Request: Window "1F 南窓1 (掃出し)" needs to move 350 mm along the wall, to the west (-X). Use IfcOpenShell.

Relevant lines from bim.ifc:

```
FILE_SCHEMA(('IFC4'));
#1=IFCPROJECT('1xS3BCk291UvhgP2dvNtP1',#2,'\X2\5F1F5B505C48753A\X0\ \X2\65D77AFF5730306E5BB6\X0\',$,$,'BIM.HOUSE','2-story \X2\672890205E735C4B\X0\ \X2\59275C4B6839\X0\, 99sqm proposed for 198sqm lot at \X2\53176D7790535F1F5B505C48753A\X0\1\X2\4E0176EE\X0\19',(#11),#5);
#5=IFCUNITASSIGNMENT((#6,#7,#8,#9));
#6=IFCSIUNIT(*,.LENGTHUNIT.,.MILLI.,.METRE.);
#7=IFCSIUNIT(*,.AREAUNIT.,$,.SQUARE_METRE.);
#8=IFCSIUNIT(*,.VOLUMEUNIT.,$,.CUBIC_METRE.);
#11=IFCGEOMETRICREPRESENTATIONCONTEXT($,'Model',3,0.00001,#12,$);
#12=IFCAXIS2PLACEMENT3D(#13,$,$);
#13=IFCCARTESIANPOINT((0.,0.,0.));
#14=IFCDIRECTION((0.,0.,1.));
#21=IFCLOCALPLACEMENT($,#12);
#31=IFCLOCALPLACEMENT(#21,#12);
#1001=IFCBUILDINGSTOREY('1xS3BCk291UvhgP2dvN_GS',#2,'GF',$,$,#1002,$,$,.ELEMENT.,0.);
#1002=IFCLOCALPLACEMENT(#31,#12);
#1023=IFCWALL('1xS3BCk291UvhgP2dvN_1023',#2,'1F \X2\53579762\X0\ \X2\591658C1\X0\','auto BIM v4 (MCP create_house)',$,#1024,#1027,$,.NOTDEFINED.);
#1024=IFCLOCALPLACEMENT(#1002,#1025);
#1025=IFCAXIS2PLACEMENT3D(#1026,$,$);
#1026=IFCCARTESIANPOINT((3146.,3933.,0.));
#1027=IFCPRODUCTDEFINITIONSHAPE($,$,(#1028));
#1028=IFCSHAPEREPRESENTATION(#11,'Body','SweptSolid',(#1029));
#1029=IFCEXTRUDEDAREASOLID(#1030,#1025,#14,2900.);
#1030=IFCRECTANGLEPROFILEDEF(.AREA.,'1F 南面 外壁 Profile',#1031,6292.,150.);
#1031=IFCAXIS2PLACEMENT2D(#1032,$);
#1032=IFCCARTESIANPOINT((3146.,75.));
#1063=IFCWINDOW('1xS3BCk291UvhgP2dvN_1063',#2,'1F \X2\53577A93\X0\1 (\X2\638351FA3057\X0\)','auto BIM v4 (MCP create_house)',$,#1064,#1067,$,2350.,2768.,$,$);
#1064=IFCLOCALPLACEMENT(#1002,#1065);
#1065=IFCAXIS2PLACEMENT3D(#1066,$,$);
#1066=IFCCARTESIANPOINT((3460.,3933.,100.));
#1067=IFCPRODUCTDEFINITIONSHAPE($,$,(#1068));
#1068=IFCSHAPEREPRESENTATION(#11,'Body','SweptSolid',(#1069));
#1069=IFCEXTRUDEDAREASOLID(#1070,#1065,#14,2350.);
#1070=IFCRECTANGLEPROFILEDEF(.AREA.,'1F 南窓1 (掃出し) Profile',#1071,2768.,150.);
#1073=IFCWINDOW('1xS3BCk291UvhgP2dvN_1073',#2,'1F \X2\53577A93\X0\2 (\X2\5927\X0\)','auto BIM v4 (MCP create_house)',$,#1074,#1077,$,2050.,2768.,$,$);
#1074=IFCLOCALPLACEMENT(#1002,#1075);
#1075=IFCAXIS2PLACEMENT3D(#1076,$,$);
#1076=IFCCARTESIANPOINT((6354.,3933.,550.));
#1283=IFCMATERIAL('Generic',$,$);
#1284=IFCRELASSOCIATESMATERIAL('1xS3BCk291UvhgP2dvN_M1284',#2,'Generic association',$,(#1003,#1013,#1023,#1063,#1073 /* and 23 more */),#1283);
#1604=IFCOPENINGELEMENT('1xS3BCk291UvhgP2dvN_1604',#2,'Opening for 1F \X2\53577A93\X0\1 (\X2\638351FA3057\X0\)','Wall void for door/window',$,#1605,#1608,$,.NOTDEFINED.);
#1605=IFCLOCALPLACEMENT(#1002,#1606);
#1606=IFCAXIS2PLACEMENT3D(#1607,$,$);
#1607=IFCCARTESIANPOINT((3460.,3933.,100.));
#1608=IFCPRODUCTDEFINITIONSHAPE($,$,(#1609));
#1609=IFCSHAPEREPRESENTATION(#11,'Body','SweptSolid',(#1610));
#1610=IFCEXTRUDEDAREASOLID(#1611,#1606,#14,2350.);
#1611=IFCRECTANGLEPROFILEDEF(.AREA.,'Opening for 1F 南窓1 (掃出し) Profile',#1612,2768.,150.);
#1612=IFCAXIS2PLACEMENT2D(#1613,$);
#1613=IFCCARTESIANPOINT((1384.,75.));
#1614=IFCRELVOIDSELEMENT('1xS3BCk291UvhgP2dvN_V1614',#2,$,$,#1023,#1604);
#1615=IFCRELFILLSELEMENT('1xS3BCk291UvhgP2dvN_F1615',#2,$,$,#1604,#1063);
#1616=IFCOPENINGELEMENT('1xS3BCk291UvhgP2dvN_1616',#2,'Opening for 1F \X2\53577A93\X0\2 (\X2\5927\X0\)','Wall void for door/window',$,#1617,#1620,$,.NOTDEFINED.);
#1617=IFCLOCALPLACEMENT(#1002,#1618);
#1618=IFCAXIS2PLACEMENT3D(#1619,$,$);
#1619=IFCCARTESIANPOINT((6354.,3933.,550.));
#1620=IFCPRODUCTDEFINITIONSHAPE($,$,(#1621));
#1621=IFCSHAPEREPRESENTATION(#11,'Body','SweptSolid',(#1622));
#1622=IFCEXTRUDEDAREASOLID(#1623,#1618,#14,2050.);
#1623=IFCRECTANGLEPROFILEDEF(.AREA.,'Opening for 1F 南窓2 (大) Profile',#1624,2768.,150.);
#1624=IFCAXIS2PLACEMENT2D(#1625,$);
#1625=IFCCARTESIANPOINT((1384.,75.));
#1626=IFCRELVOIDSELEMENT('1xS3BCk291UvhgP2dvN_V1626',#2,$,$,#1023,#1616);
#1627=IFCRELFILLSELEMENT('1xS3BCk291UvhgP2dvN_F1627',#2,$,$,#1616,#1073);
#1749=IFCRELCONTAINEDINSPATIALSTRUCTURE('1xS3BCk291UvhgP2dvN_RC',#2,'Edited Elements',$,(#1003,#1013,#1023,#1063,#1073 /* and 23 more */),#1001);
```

```python
import ifcopenshell
import ifcopenshell.api.geometry
import ifcopenshell.util.placement
import ifcopenshell.util.unit

model = ifcopenshell.open("bim.ifc")
unit_scale = ifcopenshell.util.unit.calculate_unit_scale(model)

window = model.by_guid("1xS3BCk291UvhgP2dvN_1063")
opening = window.FillsVoids[0].RelatingOpeningElement
wall = opening.VoidsElements[0].RelatingBuildingElement

wall_matrix = ifcopenshell.util.placement.get_local_placement(wall.ObjectPlacement)
shift = wall_matrix[:3, 0] * -0.35 / unit_scale
before = ifcopenshell.util.placement.get_local_placement(window.ObjectPlacement)[:3, 3].copy()

# The window is not placed relative to its opening, so move both.
for product in (opening, window):
    matrix = ifcopenshell.util.placement.get_local_placement(product.ObjectPlacement)
    matrix[:3, 3] += shift
    ifcopenshell.api.geometry.edit_object_placement(model, product=product, matrix=matrix, is_si=False)

after = ifcopenshell.util.placement.get_local_placement(window.ObjectPlacement)[:3, 3]
print("window moved by", (after - before).round(3) + 0.0)

model.write("bim_v2.ifc")
```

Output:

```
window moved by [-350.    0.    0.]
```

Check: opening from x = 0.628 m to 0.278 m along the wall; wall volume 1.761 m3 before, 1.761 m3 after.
